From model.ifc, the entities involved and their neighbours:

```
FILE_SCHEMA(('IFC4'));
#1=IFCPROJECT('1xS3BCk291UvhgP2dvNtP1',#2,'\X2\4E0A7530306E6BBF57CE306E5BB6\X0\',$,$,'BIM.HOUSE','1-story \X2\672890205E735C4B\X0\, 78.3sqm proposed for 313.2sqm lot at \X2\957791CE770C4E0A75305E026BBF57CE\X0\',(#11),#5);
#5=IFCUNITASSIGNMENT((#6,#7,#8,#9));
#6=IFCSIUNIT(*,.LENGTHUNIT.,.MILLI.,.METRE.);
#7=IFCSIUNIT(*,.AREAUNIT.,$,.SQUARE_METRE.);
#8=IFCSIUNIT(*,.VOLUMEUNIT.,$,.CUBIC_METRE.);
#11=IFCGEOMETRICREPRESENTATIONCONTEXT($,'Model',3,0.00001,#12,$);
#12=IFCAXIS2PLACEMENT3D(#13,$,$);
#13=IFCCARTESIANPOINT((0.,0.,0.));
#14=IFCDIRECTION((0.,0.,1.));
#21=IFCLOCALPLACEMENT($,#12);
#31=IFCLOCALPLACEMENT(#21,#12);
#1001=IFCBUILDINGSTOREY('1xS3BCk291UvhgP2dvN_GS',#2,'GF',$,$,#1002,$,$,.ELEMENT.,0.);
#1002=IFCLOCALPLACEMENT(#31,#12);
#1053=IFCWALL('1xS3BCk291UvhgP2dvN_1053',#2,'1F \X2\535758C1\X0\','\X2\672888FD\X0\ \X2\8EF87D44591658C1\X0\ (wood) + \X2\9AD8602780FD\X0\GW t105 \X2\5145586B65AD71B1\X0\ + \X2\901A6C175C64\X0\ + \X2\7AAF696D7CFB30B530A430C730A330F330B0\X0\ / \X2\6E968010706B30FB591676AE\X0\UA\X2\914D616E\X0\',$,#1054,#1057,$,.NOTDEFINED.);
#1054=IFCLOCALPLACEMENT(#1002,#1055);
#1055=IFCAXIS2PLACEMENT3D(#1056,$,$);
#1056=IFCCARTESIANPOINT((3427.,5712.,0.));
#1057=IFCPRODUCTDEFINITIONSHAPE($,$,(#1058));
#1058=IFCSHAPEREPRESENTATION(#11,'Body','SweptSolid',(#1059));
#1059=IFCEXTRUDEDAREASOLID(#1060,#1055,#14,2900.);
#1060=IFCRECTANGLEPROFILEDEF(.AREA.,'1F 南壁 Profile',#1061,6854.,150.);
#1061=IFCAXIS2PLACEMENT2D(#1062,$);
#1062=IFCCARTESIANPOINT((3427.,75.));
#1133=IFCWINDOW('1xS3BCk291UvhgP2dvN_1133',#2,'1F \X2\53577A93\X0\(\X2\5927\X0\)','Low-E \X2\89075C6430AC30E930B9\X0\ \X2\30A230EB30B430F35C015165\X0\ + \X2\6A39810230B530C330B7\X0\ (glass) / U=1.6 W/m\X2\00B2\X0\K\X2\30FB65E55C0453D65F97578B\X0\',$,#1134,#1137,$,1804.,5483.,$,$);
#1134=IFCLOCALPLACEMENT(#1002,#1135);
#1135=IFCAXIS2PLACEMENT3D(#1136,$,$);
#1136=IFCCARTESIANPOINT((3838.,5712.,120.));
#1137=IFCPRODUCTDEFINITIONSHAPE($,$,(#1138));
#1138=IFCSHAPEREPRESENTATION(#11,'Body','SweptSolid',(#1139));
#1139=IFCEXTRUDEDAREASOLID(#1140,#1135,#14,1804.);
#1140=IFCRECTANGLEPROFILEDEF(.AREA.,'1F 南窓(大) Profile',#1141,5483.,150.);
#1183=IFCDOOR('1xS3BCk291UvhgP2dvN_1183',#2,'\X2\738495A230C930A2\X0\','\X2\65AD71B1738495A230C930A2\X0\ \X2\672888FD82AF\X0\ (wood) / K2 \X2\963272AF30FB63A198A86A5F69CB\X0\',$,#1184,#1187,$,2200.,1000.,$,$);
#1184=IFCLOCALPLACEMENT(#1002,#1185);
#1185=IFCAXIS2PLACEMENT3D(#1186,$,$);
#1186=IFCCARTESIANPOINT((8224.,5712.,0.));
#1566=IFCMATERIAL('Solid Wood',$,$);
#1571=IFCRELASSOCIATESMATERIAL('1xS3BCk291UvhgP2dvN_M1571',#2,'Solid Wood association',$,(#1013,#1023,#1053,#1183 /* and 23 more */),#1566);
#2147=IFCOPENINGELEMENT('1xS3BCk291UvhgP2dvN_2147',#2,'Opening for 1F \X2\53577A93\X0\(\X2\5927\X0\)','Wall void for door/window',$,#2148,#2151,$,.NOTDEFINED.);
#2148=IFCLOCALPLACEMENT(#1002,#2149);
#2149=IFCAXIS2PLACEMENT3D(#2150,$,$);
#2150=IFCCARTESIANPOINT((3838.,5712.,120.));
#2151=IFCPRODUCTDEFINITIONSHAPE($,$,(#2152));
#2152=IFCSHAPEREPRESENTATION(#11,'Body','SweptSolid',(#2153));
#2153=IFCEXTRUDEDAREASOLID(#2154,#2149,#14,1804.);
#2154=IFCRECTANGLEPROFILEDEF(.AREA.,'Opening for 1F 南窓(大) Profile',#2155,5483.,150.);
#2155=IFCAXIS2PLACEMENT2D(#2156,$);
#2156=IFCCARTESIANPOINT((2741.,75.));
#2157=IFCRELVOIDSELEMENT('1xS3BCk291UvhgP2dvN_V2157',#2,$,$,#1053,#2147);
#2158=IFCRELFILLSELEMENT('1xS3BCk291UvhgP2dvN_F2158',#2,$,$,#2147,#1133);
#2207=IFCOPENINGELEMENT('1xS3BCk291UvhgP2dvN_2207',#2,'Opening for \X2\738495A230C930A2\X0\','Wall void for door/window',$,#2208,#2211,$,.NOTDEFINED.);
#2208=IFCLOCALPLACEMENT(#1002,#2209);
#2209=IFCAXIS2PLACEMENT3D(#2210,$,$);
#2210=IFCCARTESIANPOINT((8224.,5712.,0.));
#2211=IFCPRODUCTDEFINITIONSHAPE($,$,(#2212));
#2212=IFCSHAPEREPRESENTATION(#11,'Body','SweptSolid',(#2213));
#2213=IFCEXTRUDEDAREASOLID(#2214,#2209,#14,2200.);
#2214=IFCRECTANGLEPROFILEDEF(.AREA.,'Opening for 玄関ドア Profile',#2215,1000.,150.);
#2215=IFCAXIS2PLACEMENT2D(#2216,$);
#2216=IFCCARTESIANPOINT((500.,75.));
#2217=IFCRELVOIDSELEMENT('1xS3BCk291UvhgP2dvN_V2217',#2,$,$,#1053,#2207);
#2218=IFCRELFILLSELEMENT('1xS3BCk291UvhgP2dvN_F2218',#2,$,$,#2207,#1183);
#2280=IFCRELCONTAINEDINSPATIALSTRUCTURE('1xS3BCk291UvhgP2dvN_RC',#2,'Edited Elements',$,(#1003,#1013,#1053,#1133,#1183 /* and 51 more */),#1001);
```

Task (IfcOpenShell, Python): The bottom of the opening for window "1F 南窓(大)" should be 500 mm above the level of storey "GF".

```python
import numpy as np
import ifcopenshell
import ifcopenshell.api.geometry
import ifcopenshell.geom
import ifcopenshell.util.element
import ifcopenshell.util.placement
import ifcopenshell.util.shape
import ifcopenshell.util.unit

model = ifcopenshell.open("model.ifc")
unit_scale = ifcopenshell.util.unit.calculate_unit_scale(model)

window = model.by_id(1133)
opening = window.FillsVoids[0].RelatingOpeningElement
storey = ifcopenshell.util.element.get_container(window, ifc_class="IfcBuildingStorey")
level = ifcopenshell.util.placement.get_local_placement(storey.ObjectPlacement)[2, 3]

# The opening's origin need not be at the sill, so measure its lowest point.
shape = ifcopenshell.geom.create_shape(ifcopenshell.geom.settings(), opening)
bottom = ifcopenshell.util.shape.get_shape_bottom_elevation(shape, shape.geometry) / unit_scale
dz = level + 0.5 / unit_scale - bottom

shift = np.array([0.0, 0.0, dz])
# The window is not placed relative to its opening, so move both.
for product in (opening, window):
    matrix = ifcopenshell.util.placement.get_local_placement(product.ObjectPlacement)
    matrix[:3, 3] += shift
    ifcopenshell.api.geometry.edit_object_placement(model, product=product, matrix=matrix, is_si=False)

print(f"moved by {dz * unit_scale:+.3f} m")

model.write("model_edited.ifc")
```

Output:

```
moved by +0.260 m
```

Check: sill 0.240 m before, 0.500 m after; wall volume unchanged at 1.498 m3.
